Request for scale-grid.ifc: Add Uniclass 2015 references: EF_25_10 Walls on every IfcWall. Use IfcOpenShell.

First a look at what the model holds.

```python
import ifcopenshell

model = ifcopenshell.open("scale-grid.ifc")
print(model.schema)
print("classifications:", [c.Name for c in model.by_type("IfcClassification")])
for ifc_class in ("IfcDoor", "IfcRoof", "IfcStair", "IfcWall", "IfcWindow"):
    print(ifc_class, len(model.by_type(ifc_class)))
```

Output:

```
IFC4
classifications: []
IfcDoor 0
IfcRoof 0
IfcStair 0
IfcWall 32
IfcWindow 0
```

```python
import ifcopenshell
import ifcopenshell.api.classification

model = ifcopenshell.open("scale-grid.ifc")

system = ifcopenshell.api.classification.add_classification(model, classification="Uniclass 2015")

codes = {
    "IfcWall": ("EF_25_10", "Walls"),
}
for ifc_class, (code, name) in codes.items():
    products = model.by_type(ifc_class)
    ifcopenshell.api.classification.add_reference(
        model, products=products, classification=system, identification=code, name=name
    )
    print(code, len(products))

model.write("scale-grid_edited.ifc")
```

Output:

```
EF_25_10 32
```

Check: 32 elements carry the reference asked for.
